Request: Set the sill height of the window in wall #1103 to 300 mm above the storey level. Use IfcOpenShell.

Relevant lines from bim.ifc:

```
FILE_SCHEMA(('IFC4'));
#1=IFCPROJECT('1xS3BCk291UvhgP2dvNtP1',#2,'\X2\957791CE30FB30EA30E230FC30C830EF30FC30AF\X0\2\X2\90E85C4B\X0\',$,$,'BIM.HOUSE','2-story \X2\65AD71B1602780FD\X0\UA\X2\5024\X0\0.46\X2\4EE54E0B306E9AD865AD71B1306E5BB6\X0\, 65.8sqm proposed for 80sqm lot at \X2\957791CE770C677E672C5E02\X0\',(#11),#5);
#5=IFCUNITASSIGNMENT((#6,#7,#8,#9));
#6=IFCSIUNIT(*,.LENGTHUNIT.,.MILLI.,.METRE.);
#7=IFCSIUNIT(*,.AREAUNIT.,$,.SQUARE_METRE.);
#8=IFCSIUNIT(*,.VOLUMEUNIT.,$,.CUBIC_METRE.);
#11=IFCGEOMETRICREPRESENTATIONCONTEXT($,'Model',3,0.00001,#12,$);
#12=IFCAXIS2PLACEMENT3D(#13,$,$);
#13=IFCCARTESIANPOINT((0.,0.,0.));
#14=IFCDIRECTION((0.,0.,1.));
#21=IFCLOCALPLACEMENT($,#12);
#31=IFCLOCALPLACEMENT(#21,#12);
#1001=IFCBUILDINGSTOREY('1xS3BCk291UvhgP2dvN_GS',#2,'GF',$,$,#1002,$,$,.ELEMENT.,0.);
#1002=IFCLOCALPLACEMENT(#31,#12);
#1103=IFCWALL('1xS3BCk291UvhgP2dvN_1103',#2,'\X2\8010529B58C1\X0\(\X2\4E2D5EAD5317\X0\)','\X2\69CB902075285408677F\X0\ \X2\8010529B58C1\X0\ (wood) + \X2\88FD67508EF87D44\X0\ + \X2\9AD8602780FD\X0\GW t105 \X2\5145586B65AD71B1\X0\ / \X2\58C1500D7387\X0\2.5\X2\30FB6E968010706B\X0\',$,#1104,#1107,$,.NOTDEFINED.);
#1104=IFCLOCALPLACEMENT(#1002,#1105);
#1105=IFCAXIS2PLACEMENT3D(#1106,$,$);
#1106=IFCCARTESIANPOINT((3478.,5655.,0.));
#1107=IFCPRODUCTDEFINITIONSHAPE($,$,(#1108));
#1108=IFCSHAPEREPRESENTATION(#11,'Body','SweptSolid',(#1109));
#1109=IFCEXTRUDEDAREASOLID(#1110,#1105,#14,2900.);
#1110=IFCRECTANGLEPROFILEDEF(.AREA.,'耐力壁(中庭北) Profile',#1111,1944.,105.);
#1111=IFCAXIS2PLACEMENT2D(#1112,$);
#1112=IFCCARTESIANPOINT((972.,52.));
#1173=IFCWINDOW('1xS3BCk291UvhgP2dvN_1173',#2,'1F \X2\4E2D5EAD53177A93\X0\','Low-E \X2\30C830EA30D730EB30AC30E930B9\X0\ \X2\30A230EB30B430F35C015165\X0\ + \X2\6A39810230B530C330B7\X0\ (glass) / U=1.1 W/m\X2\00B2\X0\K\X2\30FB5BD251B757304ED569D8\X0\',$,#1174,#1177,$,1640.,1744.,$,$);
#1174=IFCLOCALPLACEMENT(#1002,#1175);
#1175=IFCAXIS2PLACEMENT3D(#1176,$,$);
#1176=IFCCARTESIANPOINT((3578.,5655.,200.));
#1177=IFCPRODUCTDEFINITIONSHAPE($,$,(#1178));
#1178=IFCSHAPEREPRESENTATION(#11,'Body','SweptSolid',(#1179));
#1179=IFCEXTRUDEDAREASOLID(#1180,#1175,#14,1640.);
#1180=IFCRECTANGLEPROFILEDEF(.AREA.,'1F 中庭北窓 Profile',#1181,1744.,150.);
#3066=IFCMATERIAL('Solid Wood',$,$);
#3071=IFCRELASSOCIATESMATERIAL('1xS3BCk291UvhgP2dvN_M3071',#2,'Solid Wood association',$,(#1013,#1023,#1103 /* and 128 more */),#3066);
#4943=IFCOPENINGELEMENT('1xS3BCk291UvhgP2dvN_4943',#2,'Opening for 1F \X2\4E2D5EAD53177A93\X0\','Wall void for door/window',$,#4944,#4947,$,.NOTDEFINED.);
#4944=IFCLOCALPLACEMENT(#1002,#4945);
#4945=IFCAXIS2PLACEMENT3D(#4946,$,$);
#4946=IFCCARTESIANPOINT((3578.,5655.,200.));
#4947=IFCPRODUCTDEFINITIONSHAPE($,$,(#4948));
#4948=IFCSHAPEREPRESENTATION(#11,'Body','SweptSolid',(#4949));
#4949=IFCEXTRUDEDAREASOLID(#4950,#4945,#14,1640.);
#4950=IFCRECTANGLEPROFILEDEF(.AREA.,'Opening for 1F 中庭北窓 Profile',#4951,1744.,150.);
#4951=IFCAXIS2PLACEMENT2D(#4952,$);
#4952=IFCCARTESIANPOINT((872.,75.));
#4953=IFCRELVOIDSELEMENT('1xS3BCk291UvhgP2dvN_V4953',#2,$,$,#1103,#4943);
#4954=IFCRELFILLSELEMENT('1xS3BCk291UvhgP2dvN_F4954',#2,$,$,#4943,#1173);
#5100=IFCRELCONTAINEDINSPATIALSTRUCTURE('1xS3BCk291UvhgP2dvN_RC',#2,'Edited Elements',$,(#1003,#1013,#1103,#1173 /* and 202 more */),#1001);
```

```python
import numpy as np
import ifcopenshell
import ifcopenshell.api.geometry
import ifcopenshell.geom
import ifcopenshell.util.element
import ifcopenshell.util.placement
import ifcopenshell.util.shape
import ifcopenshell.util.unit

model = ifcopenshell.open("bim.ifc")
unit_scale = ifcopenshell.util.unit.calculate_unit_scale(model)

window = model.by_guid("1xS3BCk291UvhgP2dvN_1173")
opening = window.FillsVoids[0].RelatingOpeningElement
storey = ifcopenshell.util.element.get_container(window, ifc_class="IfcBuildingStorey")
level = ifcopenshell.util.placement.get_local_placement(storey.ObjectPlacement)[2, 3]

# The opening's origin need not be at the sill, so measure its lowest point.
shape = ifcopenshell.geom.create_shape(ifcopenshell.geom.settings(), opening)
bottom = ifcopenshell.util.shape.get_shape_bottom_elevation(shape, shape.geometry) / unit_scale
dz = level + 0.3 / unit_scale - bottom

shift = np.array([0.0, 0.0, dz])
# The window is not placed relative to its opening, so move both.
for product in (opening, window):
    matrix = ifcopenshell.util.placement.get_local_placement(product.ObjectPlacement)
    matrix[:3, 3] += shift
    ifcopenshell.api.geometry.edit_object_placement(model, product=product, matrix=matrix, is_si=False)

print(f"moved by {dz * unit_scale:+.3f} m")

model.write("bim_edited.ifc")
```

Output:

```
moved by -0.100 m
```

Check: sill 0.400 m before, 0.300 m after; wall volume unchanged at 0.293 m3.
